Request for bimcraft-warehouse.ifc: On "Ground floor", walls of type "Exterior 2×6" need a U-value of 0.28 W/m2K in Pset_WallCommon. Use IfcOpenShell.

First a look at what the model holds.

```python
import ifcopenshell
import ifcopenshell.util.element

model = ifcopenshell.open("bimcraft-warehouse.ifc")
print(model.schema)
storey = next(s for s in model.by_type("IfcBuildingStorey") if s.Name == "Ground floor")
walls = [e for e in ifcopenshell.util.element.get_decomposition(storey) if e.is_a("IfcWall")]
seen = {}
for e in walls:
    element_type = ifcopenshell.util.element.get_type(e)
    key = (element_type.Name if element_type != e and element_type else None, ifcopenshell.util.element.get_pset(e, "Pset_WallCommon", "ThermalTransmittance"))
    seen[key] = seen.get(key, 0) + 1
for (name, value), count in sorted(seen.items(), key=str):
    print(count, "x", name, "|", value)
```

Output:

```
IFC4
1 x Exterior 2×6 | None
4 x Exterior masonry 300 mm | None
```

```python
import ifcopenshell
import ifcopenshell.api.pset
import ifcopenshell.util.element

model = ifcopenshell.open("bimcraft-warehouse.ifc")

storey = next(s for s in model.by_type("IfcBuildingStorey") if s.Name == "Ground floor")
walls = [e for e in ifcopenshell.util.element.get_decomposition(storey) if e.is_a("IfcWall")]

count = 0
for e in walls:
    element_type = ifcopenshell.util.element.get_type(e)
    if element_type in (None, e) or element_type.Name != "Exterior 2×6":
        continue
    # add_pset returns the element's existing set when there is one.
    pset = ifcopenshell.api.pset.add_pset(model, product=e, name="Pset_WallCommon")
    ifcopenshell.api.pset.edit_pset(model, pset=pset, properties={"ThermalTransmittance": 0.28})
    count += 1

print(count, "walls updated")

model.write("bimcraft-warehouse_updated.ifc")
```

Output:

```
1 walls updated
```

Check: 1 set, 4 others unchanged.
